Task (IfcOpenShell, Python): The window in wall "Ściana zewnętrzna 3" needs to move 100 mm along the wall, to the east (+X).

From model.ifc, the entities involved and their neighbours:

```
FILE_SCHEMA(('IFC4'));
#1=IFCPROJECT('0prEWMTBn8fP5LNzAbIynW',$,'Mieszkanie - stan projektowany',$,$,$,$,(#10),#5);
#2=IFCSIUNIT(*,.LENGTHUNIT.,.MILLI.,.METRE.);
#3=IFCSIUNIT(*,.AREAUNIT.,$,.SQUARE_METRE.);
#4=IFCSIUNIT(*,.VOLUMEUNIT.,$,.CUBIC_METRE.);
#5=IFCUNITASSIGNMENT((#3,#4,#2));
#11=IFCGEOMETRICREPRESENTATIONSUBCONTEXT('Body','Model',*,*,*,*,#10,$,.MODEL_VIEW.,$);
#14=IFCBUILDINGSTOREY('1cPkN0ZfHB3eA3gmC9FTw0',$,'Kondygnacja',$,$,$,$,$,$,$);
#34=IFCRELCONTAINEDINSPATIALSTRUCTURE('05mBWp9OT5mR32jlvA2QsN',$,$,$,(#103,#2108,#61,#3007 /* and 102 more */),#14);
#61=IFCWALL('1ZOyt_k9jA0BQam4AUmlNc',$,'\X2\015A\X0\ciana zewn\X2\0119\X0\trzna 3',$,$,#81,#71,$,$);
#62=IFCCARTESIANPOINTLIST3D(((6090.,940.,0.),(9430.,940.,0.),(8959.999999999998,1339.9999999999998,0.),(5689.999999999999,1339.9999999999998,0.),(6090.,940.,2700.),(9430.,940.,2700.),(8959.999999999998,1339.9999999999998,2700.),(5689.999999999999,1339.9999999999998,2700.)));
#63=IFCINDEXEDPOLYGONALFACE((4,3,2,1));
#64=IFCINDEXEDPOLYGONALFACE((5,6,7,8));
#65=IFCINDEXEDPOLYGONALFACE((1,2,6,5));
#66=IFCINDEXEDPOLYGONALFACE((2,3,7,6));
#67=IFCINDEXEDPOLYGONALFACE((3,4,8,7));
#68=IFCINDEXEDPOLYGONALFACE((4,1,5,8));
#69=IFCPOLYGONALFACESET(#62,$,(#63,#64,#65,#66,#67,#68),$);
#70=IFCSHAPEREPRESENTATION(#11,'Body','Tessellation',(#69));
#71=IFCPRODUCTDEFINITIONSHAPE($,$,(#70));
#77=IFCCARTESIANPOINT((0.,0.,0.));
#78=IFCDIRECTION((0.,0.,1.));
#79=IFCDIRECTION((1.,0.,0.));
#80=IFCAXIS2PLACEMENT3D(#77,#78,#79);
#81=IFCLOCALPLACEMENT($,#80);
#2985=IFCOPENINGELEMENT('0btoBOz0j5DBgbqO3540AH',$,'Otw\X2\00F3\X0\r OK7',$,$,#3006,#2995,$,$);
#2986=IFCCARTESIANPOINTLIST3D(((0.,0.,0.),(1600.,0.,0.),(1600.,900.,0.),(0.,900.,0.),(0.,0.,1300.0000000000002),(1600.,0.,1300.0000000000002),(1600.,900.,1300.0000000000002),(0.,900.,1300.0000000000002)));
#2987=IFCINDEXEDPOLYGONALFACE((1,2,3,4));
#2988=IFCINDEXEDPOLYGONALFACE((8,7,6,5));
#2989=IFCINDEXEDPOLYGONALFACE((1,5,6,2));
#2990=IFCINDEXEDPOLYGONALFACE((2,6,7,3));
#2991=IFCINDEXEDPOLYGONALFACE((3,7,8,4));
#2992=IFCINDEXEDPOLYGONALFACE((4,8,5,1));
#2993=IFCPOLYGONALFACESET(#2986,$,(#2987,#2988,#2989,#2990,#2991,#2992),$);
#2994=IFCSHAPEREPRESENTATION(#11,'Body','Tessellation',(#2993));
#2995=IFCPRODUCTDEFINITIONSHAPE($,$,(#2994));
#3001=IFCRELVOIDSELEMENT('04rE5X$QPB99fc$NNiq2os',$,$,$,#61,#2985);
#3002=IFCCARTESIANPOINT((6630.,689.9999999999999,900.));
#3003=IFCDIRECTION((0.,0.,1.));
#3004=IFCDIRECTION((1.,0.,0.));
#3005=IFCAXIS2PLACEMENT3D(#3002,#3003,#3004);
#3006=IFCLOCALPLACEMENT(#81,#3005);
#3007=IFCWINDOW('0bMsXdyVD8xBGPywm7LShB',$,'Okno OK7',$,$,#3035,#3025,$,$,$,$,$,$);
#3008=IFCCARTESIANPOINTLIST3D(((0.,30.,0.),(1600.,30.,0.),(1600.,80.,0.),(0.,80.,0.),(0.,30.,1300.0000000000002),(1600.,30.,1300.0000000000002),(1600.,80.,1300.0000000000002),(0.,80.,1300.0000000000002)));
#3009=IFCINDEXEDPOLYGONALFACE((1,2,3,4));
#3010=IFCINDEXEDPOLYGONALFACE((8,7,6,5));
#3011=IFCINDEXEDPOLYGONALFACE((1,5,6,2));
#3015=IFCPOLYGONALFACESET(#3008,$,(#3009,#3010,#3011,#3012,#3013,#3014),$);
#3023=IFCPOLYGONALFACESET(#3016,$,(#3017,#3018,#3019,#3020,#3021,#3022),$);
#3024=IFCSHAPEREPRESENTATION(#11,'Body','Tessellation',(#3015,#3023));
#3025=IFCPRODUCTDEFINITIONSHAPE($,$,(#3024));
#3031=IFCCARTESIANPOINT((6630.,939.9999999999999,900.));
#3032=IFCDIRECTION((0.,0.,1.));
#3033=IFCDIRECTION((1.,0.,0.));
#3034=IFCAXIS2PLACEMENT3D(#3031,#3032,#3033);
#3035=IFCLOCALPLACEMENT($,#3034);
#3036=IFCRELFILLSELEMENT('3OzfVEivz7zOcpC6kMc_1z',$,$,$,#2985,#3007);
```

```python
import ifcopenshell
import ifcopenshell.api.geometry
import ifcopenshell.util.placement
import ifcopenshell.util.unit

model = ifcopenshell.open("model.ifc")
unit_scale = ifcopenshell.util.unit.calculate_unit_scale(model)

window = model.by_guid("0bMsXdyVD8xBGPywm7LShB")
opening = window.FillsVoids[0].RelatingOpeningElement
wall = opening.VoidsElements[0].RelatingBuildingElement

wall_matrix = ifcopenshell.util.placement.get_local_placement(wall.ObjectPlacement)
shift = wall_matrix[:3, 0] * 0.1 / unit_scale
before = ifcopenshell.util.placement.get_local_placement(window.ObjectPlacement)[:3, 3].copy()

# The window is not placed relative to its opening, so move both.
for product in (opening, window):
    matrix = ifcopenshell.util.placement.get_local_placement(product.ObjectPlacement)
    matrix[:3, 3] += shift
    ifcopenshell.api.geometry.edit_object_placement(model, product=product, matrix=matrix, is_si=False)

after = ifcopenshell.util.placement.get_local_placement(window.ObjectPlacement)[:3, 3]
print("window moved by", (after - before).round(3) + 0.0)

model.write("model-out.ifc")
```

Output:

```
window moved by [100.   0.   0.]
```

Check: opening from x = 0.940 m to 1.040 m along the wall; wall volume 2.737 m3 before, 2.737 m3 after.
